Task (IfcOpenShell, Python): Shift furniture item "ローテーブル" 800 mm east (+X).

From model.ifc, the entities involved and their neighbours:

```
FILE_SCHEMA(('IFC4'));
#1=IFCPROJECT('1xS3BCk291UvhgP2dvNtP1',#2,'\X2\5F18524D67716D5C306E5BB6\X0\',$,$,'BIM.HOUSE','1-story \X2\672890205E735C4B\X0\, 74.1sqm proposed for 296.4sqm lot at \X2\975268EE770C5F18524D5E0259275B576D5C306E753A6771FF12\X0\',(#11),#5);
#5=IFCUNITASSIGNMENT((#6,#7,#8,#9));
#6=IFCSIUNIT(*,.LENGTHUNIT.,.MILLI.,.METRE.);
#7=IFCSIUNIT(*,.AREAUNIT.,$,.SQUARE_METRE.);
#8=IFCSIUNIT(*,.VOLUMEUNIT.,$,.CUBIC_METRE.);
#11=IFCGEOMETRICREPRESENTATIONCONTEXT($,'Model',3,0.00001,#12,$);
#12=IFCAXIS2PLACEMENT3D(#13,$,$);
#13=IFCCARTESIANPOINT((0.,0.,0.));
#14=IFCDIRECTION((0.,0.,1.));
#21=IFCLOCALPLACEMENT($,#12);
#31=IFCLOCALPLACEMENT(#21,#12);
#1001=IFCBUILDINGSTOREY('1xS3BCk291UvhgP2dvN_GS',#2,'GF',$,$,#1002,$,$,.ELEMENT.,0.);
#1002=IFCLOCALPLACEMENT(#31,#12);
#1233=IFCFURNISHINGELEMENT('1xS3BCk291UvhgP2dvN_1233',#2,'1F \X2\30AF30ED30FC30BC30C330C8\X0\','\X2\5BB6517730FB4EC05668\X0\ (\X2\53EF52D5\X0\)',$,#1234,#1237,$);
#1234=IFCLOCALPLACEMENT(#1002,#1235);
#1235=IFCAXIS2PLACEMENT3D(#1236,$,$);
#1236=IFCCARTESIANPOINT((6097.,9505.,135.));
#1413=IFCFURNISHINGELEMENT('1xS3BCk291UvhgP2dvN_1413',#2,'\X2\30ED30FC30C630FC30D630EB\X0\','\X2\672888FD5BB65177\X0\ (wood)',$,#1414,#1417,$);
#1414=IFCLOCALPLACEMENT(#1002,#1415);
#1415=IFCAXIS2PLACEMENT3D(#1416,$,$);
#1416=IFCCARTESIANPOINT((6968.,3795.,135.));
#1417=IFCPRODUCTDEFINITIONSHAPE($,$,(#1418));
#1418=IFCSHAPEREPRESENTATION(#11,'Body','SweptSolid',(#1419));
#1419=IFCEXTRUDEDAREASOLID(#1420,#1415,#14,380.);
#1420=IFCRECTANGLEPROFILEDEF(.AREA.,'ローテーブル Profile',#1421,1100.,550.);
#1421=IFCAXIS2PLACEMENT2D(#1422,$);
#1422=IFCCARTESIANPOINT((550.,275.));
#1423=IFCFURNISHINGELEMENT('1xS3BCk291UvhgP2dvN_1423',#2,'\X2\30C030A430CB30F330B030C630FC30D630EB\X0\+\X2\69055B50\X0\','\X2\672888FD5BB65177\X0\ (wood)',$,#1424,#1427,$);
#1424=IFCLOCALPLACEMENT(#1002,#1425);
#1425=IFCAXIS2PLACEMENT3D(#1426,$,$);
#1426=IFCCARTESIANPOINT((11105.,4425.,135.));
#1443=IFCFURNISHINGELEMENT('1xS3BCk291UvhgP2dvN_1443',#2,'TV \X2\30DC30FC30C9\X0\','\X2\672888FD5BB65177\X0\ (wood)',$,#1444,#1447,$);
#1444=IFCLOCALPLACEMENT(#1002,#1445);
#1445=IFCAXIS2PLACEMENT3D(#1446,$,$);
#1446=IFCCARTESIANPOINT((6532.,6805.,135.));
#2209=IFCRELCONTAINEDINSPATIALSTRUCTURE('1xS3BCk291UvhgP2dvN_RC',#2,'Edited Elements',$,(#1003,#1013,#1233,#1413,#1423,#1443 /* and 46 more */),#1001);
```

```python
import ifcopenshell
import ifcopenshell.api.geometry
import ifcopenshell.util.placement

model = ifcopenshell.open("model.ifc")

item = model.by_id(1413)
matrix = ifcopenshell.util.placement.get_local_placement(item.ObjectPlacement)
matrix[0, 3] += 800.0
ifcopenshell.api.geometry.edit_object_placement(model, product=item, matrix=matrix, is_si=False)

print(ifcopenshell.util.placement.get_local_placement(item.ObjectPlacement).round(3) + 0.0)

model.write("model_rev.ifc")
```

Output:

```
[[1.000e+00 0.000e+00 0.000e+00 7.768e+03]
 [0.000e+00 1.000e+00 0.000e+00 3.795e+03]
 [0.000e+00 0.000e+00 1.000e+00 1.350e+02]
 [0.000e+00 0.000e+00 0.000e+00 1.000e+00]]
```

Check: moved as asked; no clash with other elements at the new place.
